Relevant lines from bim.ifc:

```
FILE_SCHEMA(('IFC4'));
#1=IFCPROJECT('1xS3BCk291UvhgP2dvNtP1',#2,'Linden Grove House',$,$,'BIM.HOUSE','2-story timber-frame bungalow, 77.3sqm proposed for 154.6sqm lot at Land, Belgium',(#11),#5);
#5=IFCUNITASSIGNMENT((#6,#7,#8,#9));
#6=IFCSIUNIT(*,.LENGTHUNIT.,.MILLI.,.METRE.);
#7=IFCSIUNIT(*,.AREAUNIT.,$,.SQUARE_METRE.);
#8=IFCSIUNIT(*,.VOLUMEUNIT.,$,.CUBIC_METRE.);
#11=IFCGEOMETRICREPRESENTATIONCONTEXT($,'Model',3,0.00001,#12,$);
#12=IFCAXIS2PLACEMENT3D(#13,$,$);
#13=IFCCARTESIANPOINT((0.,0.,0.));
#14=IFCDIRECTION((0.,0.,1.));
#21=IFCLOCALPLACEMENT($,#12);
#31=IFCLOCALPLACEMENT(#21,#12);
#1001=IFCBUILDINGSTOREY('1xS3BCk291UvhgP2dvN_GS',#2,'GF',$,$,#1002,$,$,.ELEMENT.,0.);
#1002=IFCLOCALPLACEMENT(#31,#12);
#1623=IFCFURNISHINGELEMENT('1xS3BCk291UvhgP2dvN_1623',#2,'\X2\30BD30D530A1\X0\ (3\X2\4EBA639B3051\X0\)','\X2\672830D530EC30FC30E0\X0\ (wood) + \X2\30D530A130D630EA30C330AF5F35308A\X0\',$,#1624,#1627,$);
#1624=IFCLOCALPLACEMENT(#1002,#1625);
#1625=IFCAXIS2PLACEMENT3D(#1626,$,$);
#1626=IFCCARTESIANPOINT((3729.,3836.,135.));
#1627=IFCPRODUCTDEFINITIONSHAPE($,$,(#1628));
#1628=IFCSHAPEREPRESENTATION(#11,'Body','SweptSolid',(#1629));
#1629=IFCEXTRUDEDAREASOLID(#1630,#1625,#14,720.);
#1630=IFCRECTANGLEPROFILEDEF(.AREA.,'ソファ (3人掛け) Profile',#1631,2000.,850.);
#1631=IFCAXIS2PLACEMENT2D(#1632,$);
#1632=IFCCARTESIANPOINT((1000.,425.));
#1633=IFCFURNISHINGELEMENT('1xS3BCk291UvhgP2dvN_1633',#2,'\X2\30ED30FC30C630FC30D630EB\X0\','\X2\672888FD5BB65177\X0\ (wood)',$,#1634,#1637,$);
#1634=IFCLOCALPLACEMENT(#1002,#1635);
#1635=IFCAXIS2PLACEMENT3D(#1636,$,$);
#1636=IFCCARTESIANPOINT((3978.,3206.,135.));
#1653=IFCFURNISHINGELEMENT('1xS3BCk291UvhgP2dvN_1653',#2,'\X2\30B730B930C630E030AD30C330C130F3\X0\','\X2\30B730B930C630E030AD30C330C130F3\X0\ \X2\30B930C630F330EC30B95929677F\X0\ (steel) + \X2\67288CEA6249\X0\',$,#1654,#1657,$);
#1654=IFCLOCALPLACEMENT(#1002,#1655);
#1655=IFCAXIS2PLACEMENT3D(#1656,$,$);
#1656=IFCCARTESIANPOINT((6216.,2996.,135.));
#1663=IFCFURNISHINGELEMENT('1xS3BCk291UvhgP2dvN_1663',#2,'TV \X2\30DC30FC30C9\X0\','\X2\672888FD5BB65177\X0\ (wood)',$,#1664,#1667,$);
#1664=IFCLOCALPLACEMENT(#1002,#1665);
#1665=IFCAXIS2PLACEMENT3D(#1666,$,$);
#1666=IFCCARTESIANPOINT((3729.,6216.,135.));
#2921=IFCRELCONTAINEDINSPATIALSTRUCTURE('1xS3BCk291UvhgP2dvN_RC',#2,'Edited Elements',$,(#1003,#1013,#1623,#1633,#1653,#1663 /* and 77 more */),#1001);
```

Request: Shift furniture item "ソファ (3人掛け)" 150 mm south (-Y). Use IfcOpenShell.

```python
import ifcopenshell
import ifcopenshell.api.geometry
import ifcopenshell.util.placement
import ifcopenshell.util.unit

model = ifcopenshell.open("bim.ifc")
unit_scale = ifcopenshell.util.unit.calculate_unit_scale(model)

item = model.by_guid("1xS3BCk291UvhgP2dvN_1623")
matrix = ifcopenshell.util.placement.get_local_placement(item.ObjectPlacement)
matrix[1, 3] -= 0.15 / unit_scale
ifcopenshell.api.geometry.edit_object_placement(model, product=item, matrix=matrix, is_si=False)

print(ifcopenshell.util.placement.get_local_placement(item.ObjectPlacement).round(3) + 0.0)

model.write("bim_rev.ifc")
```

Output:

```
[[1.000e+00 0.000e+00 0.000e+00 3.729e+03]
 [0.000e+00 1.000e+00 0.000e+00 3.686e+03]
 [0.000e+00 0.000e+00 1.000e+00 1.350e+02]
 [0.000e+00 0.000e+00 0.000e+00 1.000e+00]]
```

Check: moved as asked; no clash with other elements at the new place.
